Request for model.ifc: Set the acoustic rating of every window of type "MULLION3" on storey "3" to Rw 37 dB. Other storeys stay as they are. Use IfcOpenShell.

First a look at what the model holds.

```python
import ifcopenshell
import ifcopenshell.util.element

model = ifcopenshell.open("model.ifc")
print(model.schema)
storey = next(s for s in model.by_type("IfcBuildingStorey") if s.Name == "3")
windows = [e for e in ifcopenshell.util.element.get_decomposition(storey) if e.is_a("IfcWindow")]
seen = {}
for e in windows:
    element_type = ifcopenshell.util.element.get_type(e)
    key = (element_type.Name if element_type != e and element_type else None, ifcopenshell.util.element.get_pset(e, "Pset_WindowCommon", "AcousticRating"))
    seen[key] = seen.get(key, 0) + 1
for (name, value), count in sorted(seen.items(), key=str):
    print(count, "x", name, "|", value)
```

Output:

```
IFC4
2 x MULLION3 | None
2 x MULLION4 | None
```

```python
import ifcopenshell
import ifcopenshell.api.pset
import ifcopenshell.util.element

model = ifcopenshell.open("model.ifc")

storey = next(s for s in model.by_type("IfcBuildingStorey") if s.Name == "3")
windows = [e for e in ifcopenshell.util.element.get_decomposition(storey) if e.is_a("IfcWindow")]

count = 0
for e in windows:
    element_type = ifcopenshell.util.element.get_type(e)
    if element_type in (None, e) or element_type.Name != "MULLION3":
        continue
    # add_pset returns the element's existing set when there is one.
    pset = ifcopenshell.api.pset.add_pset(model, product=e, name="Pset_WindowCommon")
    ifcopenshell.api.pset.edit_pset(model, pset=pset, properties={"AcousticRating": "Rw 37 dB"})
    count += 1

print(count, "windows updated")

model.write("model-out.ifc")
```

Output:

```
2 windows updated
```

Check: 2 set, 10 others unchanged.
